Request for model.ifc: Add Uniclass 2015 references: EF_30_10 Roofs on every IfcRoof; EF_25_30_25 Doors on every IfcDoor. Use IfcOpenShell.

First a look at what the model holds.

```python
import ifcopenshell

model = ifcopenshell.open("model.ifc")
print(model.schema)
print("classifications:", [c.Name for c in model.by_type("IfcClassification")])
for ifc_class in ("IfcDoor", "IfcRoof", "IfcStair", "IfcWall", "IfcWindow"):
    print(ifc_class, len(model.by_type(ifc_class)))
```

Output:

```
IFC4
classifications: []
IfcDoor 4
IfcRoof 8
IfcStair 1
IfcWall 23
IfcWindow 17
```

```python
import ifcopenshell
import ifcopenshell.api.classification

model = ifcopenshell.open("model.ifc")

system = ifcopenshell.api.classification.add_classification(model, classification="Uniclass 2015")

codes = {
    "IfcRoof": ("EF_30_10", "Roofs"),
    "IfcDoor": ("EF_25_30_25", "Doors"),
}
for ifc_class, (code, name) in codes.items():
    products = model.by_type(ifc_class)
    ifcopenshell.api.classification.add_reference(
        model, products=products, classification=system, identification=code, name=name
    )
    print(code, len(products))

model.write("model_rev.ifc")
```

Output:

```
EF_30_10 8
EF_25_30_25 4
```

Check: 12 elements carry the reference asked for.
